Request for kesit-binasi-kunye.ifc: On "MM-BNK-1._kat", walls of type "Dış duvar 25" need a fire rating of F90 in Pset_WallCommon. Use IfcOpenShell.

First a look at what the model holds.

```python
import ifcopenshell
import ifcopenshell.util.element

model = ifcopenshell.open("kesit-binasi-kunye.ifc")
print(model.schema)
storey = next(s for s in model.by_type("IfcBuildingStorey") if s.Name == "MM-BNK-1._kat")
walls = [e for e in ifcopenshell.util.element.get_decomposition(storey) if e.is_a("IfcWall")]
seen = {}
for e in walls:
    element_type = ifcopenshell.util.element.get_type(e)
    key = (element_type.Name if element_type != e and element_type else None, ifcopenshell.util.element.get_pset(e, "Pset_WallCommon", "FireRating"))
    seen[key] = seen.get(key, 0) + 1
for (name, value), count in sorted(seen.items(), key=str):
    print(count, "x", name, "|", value)
```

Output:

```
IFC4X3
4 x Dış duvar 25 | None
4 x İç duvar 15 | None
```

```python
import ifcopenshell
import ifcopenshell.api.pset
import ifcopenshell.util.element

model = ifcopenshell.open("kesit-binasi-kunye.ifc")

storey = next(s for s in model.by_type("IfcBuildingStorey") if s.Name == "MM-BNK-1._kat")
walls = [e for e in ifcopenshell.util.element.get_decomposition(storey) if e.is_a("IfcWall")]

count = 0
for e in walls:
    element_type = ifcopenshell.util.element.get_type(e)
    if element_type in (None, e) or element_type.Name != "Dış duvar 25":
        continue
    # add_pset returns the element's existing set when there is one.
    pset = ifcopenshell.api.pset.add_pset(model, product=e, name="Pset_WallCommon")
    ifcopenshell.api.pset.edit_pset(model, pset=pset, properties={"FireRating": "F90"})
    count += 1

print(count, "walls updated")

model.write("kesit-binasi-kunye_rev.ifc")
```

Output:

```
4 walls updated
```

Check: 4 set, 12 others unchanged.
